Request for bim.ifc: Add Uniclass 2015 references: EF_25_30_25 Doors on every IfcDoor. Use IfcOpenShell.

First a look at what the model holds.

```python
import ifcopenshell

model = ifcopenshell.open("bim.ifc")
print(model.schema)
print("classifications:", [c.Name for c in model.by_type("IfcClassification")])
for ifc_class in ("IfcDoor", "IfcRoof", "IfcStair", "IfcWall", "IfcWindow"):
    print(ifc_class, len(model.by_type(ifc_class)))
```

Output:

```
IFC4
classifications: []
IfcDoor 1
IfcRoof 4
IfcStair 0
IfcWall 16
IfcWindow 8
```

```python
import ifcopenshell
import ifcopenshell.api.classification

model = ifcopenshell.open("bim.ifc")

system = ifcopenshell.api.classification.add_classification(model, classification="Uniclass 2015")

codes = {
    "IfcDoor": ("EF_25_30_25", "Doors"),
}
for ifc_class, (code, name) in codes.items():
    products = model.by_type(ifc_class)
    ifcopenshell.api.classification.add_reference(
        model, products=products, classification=system, identification=code, name=name
    )
    print(code, len(products))

model.write("bim_rev.ifc")
```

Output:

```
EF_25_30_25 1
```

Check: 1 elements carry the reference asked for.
